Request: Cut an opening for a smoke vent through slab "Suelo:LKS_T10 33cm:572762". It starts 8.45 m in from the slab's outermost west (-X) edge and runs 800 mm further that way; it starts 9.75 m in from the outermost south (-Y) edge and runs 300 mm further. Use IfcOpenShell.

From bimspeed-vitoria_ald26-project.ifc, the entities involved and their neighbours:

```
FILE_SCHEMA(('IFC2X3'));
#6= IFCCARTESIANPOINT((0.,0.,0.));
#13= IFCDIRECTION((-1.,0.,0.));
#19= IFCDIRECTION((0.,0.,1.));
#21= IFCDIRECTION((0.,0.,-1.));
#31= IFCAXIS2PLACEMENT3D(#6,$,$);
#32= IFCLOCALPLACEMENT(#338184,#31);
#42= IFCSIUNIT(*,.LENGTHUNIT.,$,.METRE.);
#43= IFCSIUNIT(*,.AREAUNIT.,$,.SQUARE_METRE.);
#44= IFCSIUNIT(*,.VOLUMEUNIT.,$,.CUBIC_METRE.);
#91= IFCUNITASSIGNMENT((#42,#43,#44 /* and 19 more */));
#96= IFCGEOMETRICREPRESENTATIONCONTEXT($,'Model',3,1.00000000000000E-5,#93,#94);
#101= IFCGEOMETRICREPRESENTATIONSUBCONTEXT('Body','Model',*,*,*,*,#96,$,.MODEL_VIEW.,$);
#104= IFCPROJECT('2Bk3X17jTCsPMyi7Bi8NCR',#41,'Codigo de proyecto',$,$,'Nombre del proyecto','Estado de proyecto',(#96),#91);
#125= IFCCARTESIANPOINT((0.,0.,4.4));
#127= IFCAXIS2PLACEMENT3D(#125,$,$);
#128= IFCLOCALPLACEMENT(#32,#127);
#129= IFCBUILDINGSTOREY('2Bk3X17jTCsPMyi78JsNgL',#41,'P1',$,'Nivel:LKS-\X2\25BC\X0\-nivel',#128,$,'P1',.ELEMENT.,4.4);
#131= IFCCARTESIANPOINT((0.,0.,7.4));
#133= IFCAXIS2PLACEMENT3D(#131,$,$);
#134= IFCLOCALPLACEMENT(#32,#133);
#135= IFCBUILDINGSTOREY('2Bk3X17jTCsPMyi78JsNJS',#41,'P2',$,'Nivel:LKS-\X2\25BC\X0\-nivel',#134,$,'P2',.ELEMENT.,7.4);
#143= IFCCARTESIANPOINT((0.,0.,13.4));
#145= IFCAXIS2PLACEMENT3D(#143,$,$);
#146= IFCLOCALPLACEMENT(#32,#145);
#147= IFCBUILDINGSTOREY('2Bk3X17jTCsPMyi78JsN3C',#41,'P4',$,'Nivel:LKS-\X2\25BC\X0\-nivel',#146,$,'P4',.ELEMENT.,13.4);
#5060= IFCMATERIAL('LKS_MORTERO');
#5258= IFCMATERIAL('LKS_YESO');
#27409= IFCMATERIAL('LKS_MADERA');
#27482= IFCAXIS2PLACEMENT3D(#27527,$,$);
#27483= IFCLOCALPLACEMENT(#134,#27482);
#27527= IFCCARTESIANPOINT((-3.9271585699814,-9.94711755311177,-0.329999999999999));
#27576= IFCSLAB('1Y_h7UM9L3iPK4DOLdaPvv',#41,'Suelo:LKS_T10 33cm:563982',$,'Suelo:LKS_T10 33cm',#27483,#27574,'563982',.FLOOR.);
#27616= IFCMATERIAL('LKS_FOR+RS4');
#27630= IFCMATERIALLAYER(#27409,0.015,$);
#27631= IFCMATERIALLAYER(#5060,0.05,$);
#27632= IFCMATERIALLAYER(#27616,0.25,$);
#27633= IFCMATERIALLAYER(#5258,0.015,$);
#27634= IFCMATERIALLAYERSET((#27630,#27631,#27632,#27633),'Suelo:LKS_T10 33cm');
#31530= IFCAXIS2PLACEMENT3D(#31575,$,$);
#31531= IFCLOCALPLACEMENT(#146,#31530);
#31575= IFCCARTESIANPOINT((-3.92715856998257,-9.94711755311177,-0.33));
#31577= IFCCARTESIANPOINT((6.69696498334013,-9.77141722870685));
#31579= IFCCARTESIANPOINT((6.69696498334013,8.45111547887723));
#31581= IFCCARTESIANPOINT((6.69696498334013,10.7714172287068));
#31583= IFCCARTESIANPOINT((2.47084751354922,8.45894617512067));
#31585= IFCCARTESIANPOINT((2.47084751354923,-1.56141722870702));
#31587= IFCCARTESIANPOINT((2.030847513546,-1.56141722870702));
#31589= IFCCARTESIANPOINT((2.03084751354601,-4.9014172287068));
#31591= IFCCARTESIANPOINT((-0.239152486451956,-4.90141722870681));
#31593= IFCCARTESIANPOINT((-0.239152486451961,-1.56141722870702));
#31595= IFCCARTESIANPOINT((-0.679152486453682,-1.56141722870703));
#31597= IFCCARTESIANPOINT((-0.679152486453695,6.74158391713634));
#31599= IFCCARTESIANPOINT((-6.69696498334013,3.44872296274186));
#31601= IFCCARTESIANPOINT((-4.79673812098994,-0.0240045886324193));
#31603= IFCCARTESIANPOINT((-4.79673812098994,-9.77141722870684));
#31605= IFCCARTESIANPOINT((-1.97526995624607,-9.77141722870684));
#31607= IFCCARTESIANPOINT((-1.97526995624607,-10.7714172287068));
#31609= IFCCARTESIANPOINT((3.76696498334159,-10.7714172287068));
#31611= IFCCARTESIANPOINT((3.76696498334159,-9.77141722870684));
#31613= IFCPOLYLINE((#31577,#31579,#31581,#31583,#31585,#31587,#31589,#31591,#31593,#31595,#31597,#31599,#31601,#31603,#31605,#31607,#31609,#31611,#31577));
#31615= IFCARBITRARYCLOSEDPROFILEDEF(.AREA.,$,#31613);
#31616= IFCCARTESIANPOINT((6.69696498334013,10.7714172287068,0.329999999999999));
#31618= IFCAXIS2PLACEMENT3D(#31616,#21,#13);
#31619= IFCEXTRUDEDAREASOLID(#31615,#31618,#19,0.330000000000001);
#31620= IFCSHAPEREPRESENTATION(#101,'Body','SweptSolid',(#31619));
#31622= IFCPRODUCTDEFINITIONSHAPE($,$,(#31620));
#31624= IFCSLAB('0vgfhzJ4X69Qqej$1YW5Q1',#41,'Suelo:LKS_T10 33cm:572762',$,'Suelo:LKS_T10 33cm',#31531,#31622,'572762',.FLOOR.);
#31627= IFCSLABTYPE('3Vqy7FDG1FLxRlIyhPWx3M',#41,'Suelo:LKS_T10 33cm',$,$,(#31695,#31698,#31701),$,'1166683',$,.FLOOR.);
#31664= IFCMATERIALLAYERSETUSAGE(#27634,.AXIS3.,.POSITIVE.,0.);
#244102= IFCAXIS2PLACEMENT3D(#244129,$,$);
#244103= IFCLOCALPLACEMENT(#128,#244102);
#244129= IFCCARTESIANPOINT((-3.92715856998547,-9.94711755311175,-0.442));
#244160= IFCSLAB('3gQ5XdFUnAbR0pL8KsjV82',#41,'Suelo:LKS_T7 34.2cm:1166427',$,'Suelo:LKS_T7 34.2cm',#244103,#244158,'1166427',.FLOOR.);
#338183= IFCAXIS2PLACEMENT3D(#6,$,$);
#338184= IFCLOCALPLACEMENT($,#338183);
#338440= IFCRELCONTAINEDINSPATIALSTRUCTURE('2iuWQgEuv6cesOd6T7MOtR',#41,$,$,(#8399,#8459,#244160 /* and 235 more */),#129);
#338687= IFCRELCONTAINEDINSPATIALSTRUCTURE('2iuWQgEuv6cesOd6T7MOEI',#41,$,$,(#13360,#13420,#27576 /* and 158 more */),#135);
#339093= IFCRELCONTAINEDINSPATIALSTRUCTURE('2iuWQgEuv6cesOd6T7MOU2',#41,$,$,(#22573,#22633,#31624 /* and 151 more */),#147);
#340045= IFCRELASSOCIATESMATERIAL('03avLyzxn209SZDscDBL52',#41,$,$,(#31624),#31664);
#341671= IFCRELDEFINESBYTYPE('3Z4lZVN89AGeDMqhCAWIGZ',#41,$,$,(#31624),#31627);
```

```python
import numpy as np
import ifcopenshell
import ifcopenshell.api.feature
import ifcopenshell.api.geometry
import ifcopenshell.api.root
import ifcopenshell.geom
import ifcopenshell.util.placement
import ifcopenshell.util.representation
import ifcopenshell.util.shape
import ifcopenshell.util.unit

model = ifcopenshell.open("bimspeed-vitoria_ald26-project.ifc")
unit_scale = ifcopenshell.util.unit.calculate_unit_scale(model)
settings = ifcopenshell.geom.settings()


def volume(element):
    """Net volume in cubic metres, openings subtracted."""
    shape = ifcopenshell.geom.create_shape(settings, element)
    return ifcopenshell.util.shape.get_volume(shape.geometry)


slab = model.by_id(31624)
before = volume(slab)

# Extent in the slab's own axes, in metres. The edges named are its -X and -Y sides.
slab_shape = ifcopenshell.geom.create_shape(settings, slab)
vertices = ifcopenshell.util.shape.get_vertices(slab_shape.geometry)
x_min, y_min, bottom = vertices.min(axis=0)
top = vertices[:, 2].max()

opening = ifcopenshell.api.root.create_entity(model, ifc_class="IfcOpeningElement", name="Smoke vent opening")
context = ifcopenshell.util.representation.get_context(model, "Model", "Body", "MODEL_VIEW")
width, depth = 0.8, 0.3
outline = [(0.0, 0.0), (width, 0.0), (width, depth), (0.0, depth), (0.0, 0.0)]
# Overshoot both faces by 50 mm so the cut is clean.
shape = ifcopenshell.api.geometry.add_slab_representation(
    model, context=context, depth=top - bottom + 0.1, polyline=outline
)
ifcopenshell.api.geometry.assign_representation(model, product=opening, representation=shape)

matrix = ifcopenshell.util.placement.get_local_placement(slab.ObjectPlacement)
matrix[:, 3] = matrix @ np.append(np.array([x_min + 8.45, y_min + 9.75, bottom - 0.05]) / unit_scale, 1.0)
ifcopenshell.api.geometry.edit_object_placement(model, product=opening, matrix=matrix, is_si=False)
ifcopenshell.api.feature.add_feature(model, feature=opening, element=slab)

after = volume(slab)

print(f"slab volume {before:.3f} -> {after:.3f} m3")

model.write("bimspeed-vitoria_ald26-project_updated.ifc")
```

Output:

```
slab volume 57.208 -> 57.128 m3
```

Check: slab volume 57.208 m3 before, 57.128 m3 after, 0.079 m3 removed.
